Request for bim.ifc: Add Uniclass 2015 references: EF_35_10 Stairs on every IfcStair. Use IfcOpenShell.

First a look at what the model holds.

```python
import ifcopenshell

model = ifcopenshell.open("bim.ifc")
print(model.schema)
print("classifications:", [c.Name for c in model.by_type("IfcClassification")])
for ifc_class in ("IfcDoor", "IfcRoof", "IfcStair", "IfcWall", "IfcWindow"):
    print(ifc_class, len(model.by_type(ifc_class)))
```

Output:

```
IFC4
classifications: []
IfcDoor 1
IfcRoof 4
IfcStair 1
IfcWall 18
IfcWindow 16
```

```python
import ifcopenshell
import ifcopenshell.api.classification

model = ifcopenshell.open("bim.ifc")

system = ifcopenshell.api.classification.add_classification(model, classification="Uniclass 2015")

codes = {
    "IfcStair": ("EF_35_10", "Stairs"),
}
for ifc_class, (code, name) in codes.items():
    products = model.by_type(ifc_class)
    ifcopenshell.api.classification.add_reference(
        model, products=products, classification=system, identification=code, name=name
    )
    print(code, len(products))

model.write("bim_edited.ifc")
```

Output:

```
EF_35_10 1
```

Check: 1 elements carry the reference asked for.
